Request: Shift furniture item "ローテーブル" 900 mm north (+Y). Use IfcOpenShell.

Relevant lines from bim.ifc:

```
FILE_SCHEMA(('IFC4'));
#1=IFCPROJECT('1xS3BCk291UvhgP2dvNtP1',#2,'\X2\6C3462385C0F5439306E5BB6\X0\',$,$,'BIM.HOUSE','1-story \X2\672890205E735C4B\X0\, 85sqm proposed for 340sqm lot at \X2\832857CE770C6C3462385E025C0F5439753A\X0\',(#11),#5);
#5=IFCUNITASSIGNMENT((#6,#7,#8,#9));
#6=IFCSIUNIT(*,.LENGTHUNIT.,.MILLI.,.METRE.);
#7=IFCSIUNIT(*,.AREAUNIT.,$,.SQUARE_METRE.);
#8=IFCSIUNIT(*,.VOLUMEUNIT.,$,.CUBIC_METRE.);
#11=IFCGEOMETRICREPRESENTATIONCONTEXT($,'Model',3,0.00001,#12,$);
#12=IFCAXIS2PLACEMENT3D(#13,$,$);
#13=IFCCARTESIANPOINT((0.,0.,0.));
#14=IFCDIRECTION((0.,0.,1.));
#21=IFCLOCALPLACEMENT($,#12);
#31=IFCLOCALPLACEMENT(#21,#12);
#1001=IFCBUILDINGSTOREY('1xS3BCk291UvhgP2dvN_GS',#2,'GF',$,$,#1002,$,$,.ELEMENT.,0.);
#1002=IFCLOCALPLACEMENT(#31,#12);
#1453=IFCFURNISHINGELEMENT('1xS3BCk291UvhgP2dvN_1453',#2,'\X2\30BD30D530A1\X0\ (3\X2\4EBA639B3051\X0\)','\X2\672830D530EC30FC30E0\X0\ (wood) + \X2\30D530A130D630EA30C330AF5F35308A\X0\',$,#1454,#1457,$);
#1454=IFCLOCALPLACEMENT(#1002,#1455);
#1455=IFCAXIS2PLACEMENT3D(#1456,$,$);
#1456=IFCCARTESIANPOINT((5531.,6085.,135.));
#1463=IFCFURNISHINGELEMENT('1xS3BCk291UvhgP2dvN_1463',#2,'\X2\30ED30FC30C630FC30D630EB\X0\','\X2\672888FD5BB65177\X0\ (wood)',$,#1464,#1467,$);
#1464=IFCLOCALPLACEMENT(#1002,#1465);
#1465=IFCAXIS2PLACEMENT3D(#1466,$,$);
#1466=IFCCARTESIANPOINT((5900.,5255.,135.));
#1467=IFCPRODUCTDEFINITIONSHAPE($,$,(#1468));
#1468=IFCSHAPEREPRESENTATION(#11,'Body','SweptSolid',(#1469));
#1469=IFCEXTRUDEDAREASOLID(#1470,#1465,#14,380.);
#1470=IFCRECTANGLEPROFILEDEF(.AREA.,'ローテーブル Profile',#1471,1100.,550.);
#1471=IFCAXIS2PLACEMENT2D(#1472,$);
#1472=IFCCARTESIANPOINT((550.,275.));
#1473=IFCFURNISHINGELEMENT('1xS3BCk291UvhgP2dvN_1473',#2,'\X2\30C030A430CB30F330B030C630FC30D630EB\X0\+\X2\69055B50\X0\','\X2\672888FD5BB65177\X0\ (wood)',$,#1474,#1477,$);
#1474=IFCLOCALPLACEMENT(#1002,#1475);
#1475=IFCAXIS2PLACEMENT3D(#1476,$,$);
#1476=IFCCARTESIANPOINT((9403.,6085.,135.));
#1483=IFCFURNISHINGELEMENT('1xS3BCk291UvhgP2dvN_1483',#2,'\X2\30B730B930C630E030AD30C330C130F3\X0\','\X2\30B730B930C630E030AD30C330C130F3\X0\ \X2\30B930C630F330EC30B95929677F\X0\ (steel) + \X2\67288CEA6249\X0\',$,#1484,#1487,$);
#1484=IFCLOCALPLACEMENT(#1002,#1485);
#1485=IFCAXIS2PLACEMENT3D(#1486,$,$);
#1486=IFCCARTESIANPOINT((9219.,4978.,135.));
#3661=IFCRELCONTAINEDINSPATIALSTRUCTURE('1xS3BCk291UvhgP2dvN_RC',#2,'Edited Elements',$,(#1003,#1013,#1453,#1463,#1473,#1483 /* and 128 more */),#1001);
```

```python
import ifcopenshell
import ifcopenshell.api.geometry
import ifcopenshell.util.placement
import ifcopenshell.util.unit

model = ifcopenshell.open("bim.ifc")
unit_scale = ifcopenshell.util.unit.calculate_unit_scale(model)

item = model.by_id(1463)
matrix = ifcopenshell.util.placement.get_local_placement(item.ObjectPlacement)
matrix[1, 3] += 0.9 / unit_scale
ifcopenshell.api.geometry.edit_object_placement(model, product=item, matrix=matrix, is_si=False)

print(ifcopenshell.util.placement.get_local_placement(item.ObjectPlacement).round(3) + 0.0)

model.write("bim_v2.ifc")
```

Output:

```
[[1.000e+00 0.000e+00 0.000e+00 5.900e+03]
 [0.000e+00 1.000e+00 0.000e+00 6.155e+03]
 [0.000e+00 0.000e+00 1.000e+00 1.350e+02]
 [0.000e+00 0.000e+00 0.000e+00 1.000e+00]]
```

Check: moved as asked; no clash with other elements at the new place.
